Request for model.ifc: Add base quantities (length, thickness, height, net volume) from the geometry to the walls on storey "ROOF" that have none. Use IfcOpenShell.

First a look at what the model holds.

```python
import ifcopenshell
import ifcopenshell.util.element
import ifcopenshell.util.unit

model = ifcopenshell.open("model.ifc")
print(model.schema)
for unit_type in ("LENGTHUNIT", "AREAUNIT", "VOLUMEUNIT"):
    print(unit_type, ifcopenshell.util.unit.calculate_unit_scale(model, unit_type))
storey = next(s for s in model.by_type("IfcBuildingStorey") if s.Name == "ROOF")
walls = [e for e in ifcopenshell.util.element.get_decomposition(storey) if e.is_a("IfcWall")]
for e in sorted(walls, key=lambda e: e.id()):
    print(e.id(), e.is_a(), e.Name, list(ifcopenshell.util.element.get_psets(e, qtos_only=True)), sep=" | ")
```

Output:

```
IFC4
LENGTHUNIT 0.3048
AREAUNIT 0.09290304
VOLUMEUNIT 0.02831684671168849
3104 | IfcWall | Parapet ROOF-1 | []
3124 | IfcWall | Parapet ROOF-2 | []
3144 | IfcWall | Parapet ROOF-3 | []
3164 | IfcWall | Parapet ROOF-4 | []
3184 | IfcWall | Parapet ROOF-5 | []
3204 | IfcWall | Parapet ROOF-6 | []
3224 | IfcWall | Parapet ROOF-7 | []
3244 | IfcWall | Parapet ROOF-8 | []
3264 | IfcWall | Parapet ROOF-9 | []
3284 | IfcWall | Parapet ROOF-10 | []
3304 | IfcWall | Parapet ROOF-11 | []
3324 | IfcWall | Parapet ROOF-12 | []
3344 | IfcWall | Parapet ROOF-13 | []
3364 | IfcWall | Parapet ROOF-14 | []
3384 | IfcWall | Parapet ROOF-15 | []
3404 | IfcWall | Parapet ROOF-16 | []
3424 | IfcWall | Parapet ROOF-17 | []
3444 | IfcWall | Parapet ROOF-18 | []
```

```python
import ifcopenshell
import ifcopenshell.api.pset
import ifcopenshell.geom
import ifcopenshell.util.element
import ifcopenshell.util.shape
import ifcopenshell.util.unit

model = ifcopenshell.open("model.ifc")
unit_scale = ifcopenshell.util.unit.calculate_unit_scale(model)
volume_scale = ifcopenshell.util.unit.calculate_unit_scale(model, "VOLUMEUNIT")
settings = ifcopenshell.geom.settings()

storey = next(s for s in model.by_type("IfcBuildingStorey") if s.Name == "ROOF")
walls = [e for e in ifcopenshell.util.element.get_decomposition(storey) if e.is_a("IfcWall")]

for e in sorted(walls, key=lambda e: e.id()):
    if ifcopenshell.util.element.get_psets(e, qtos_only=True, should_inherit=False):
        continue
    # Geometry comes back in metres, in the element's own axes.
    shape = ifcopenshell.geom.create_shape(settings, e)
    values = {
        "Length": ifcopenshell.util.shape.get_x(shape.geometry) / unit_scale,
        "Width": ifcopenshell.util.shape.get_y(shape.geometry) / unit_scale,
        "Height": ifcopenshell.util.shape.get_z(shape.geometry) / unit_scale,
        "NetVolume": ifcopenshell.util.shape.get_volume(shape.geometry) / volume_scale,
    }
    qto = ifcopenshell.api.pset.add_qto(model, product=e, name="Qto_WallBaseQuantities")
    ifcopenshell.api.pset.edit_qto(model, qto=qto, properties=values)
    print(e.id(), {k: round(v, 3) for k, v in values.items()})

model.write("model_rev.ifc")
```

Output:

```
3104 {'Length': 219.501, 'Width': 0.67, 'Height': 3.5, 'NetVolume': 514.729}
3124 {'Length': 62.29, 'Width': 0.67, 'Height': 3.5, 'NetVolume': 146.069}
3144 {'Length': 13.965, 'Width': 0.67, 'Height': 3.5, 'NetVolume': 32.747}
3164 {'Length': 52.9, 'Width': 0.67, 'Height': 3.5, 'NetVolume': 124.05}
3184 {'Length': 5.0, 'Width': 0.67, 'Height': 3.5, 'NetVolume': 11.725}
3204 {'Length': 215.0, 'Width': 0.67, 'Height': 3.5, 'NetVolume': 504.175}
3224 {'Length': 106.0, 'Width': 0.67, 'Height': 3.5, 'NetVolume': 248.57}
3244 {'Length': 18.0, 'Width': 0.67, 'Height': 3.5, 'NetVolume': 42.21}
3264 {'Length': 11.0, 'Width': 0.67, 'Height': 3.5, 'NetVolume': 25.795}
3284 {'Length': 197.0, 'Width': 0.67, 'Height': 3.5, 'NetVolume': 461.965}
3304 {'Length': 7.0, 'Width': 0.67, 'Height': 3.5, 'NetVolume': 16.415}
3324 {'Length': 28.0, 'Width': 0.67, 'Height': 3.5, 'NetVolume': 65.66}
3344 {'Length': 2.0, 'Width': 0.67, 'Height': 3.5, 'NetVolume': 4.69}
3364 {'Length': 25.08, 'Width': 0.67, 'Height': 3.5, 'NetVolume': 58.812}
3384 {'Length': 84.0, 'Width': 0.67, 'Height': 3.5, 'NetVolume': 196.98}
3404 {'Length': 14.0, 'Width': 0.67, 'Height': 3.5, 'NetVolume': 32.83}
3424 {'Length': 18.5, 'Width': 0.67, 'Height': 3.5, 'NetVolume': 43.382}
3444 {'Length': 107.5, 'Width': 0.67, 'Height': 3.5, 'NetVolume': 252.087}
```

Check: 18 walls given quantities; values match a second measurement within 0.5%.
